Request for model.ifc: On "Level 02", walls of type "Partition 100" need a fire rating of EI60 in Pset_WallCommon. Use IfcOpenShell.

First a look at what the model holds.

```python
import ifcopenshell
import ifcopenshell.util.element

model = ifcopenshell.open("model.ifc")
print(model.schema)
storey = next(s for s in model.by_type("IfcBuildingStorey") if s.Name == "Level 02")
walls = [e for e in ifcopenshell.util.element.get_decomposition(storey) if e.is_a("IfcWall")]
seen = {}
for e in walls:
    element_type = ifcopenshell.util.element.get_type(e)
    key = (element_type.Name if element_type != e and element_type else None, ifcopenshell.util.element.get_pset(e, "Pset_WallCommon", "FireRating"))
    seen[key] = seen.get(key, 0) + 1
for (name, value), count in sorted(seen.items(), key=str):
    print(count, "x", name, "|", value)
```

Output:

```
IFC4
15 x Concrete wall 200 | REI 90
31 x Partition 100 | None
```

```python
import ifcopenshell
import ifcopenshell.api.pset
import ifcopenshell.util.element

model = ifcopenshell.open("model.ifc")

storey = next(s for s in model.by_type("IfcBuildingStorey") if s.Name == "Level 02")
walls = [e for e in ifcopenshell.util.element.get_decomposition(storey) if e.is_a("IfcWall")]

count = 0
for e in walls:
    element_type = ifcopenshell.util.element.get_type(e)
    if element_type in (None, e) or element_type.Name != "Partition 100":
        continue
    # add_pset returns the element's existing set when there is one.
    pset = ifcopenshell.api.pset.add_pset(model, product=e, name="Pset_WallCommon")
    ifcopenshell.api.pset.edit_pset(model, pset=pset, properties={"FireRating": "EI60"})
    count += 1

print(count, "walls updated")

model.write("model_edited.ifc")
```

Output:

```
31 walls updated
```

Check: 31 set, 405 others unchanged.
